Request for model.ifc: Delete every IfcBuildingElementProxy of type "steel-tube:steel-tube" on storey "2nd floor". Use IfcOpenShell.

First a look at what the model holds.

```python
import ifcopenshell
import ifcopenshell.util.element

model = ifcopenshell.open("model.ifc")
print(model.schema)
storey = next(s for s in model.by_type("IfcBuildingStorey") if s.Name == "2nd floor")
proxies = [e for e in ifcopenshell.util.element.get_decomposition(storey) if e.is_a("IfcBuildingElementProxy")]
seen = {}
for e in proxies:
    element_type = ifcopenshell.util.element.get_type(e)
    name = element_type.Name if element_type not in (None, e) else None
    seen[name] = seen.get(name, 0) + 1
for name, count in sorted(seen.items(), key=str):
    print(count, "x", name)
```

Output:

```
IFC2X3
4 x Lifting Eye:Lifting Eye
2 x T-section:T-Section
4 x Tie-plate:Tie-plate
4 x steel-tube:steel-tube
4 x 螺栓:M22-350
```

```python
import ifcopenshell
import ifcopenshell.api.root
import ifcopenshell.util.element

model = ifcopenshell.open("model.ifc")

storey = next(s for s in model.by_type("IfcBuildingStorey") if s.Name == "2nd floor")
proxies = [e for e in ifcopenshell.util.element.get_decomposition(storey) if e.is_a("IfcBuildingElementProxy")]
targets = [e for e in proxies if (t := ifcopenshell.util.element.get_type(e)) not in (None, e) and t.Name == "steel-tube:steel-tube"]

for e in targets:
    ifcopenshell.api.root.remove_product(model, product=e)
print(len(targets), "removed")

model.write("model_edited.ifc")
```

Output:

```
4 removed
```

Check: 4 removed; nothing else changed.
